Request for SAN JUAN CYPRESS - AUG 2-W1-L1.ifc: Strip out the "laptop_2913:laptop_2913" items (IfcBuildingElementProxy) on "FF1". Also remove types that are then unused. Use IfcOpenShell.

First a look at what the model holds.

```python
import ifcopenshell
import ifcopenshell.util.element

model = ifcopenshell.open("SAN JUAN CYPRESS - AUG 2-W1-L1.ifc")
print(model.schema)
storey = next(s for s in model.by_type("IfcBuildingStorey") if s.Name == "FF1")
proxies = [e for e in ifcopenshell.util.element.get_decomposition(storey) if e.is_a("IfcBuildingElementProxy")]
seen = {}
for e in proxies:
    element_type = ifcopenshell.util.element.get_type(e)
    name = element_type.Name if element_type not in (None, e) else None
    seen[name] = seen.get(name, 0) + 1
for name, count in sorted(seen.items(), key=str):
    print(count, "x", name)
```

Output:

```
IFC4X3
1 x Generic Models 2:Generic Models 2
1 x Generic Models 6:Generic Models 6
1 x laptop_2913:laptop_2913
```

```python
import ifcopenshell
import ifcopenshell.api.root
import ifcopenshell.util.element

model = ifcopenshell.open("SAN JUAN CYPRESS - AUG 2-W1-L1.ifc")

storey = next(s for s in model.by_type("IfcBuildingStorey") if s.Name == "FF1")
proxies = [e for e in ifcopenshell.util.element.get_decomposition(storey) if e.is_a("IfcBuildingElementProxy")]
targets = [e for e in proxies if (t := ifcopenshell.util.element.get_type(e)) not in (None, e) and t.Name == "laptop_2913:laptop_2913"]
types = {ifcopenshell.util.element.get_type(e) for e in targets} - {None, *targets}

for e in targets:
    ifcopenshell.api.root.remove_product(model, product=e)
print(len(targets), "removed")

unused = [t for t in types if not ifcopenshell.util.element.get_types(t)]
for t in unused:
    ifcopenshell.api.root.remove_product(model, product=t)
print(len(unused), "unused types removed")

model.write("SAN JUAN CYPRESS - AUG 2-W1-L1-out.ifc")
```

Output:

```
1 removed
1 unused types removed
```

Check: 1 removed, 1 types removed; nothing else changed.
